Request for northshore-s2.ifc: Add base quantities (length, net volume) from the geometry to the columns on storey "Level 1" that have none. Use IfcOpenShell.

First a look at what the model holds.

```python
import ifcopenshell
import ifcopenshell.util.element
import ifcopenshell.util.unit

model = ifcopenshell.open("northshore-s2.ifc")
print(model.schema)
for unit_type in ("LENGTHUNIT", "AREAUNIT", "VOLUMEUNIT"):
    print(unit_type, ifcopenshell.util.unit.calculate_unit_scale(model, unit_type))
storey = next(s for s in model.by_type("IfcBuildingStorey") if s.Name == "Level 1")
columns = [e for e in ifcopenshell.util.element.get_decomposition(storey) if e.is_a("IfcColumn")]
for e in sorted(columns, key=lambda e: e.id()):
    print(e.id(), e.is_a(), e.Name, list(ifcopenshell.util.element.get_psets(e, qtos_only=True)), sep=" | ")
```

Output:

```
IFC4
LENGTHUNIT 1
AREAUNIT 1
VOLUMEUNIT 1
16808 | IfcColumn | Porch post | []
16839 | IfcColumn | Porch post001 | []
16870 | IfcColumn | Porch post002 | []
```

```python
import ifcopenshell
import ifcopenshell.api.pset
import ifcopenshell.geom
import ifcopenshell.util.element
import ifcopenshell.util.shape
import ifcopenshell.util.unit

model = ifcopenshell.open("northshore-s2.ifc")
unit_scale = ifcopenshell.util.unit.calculate_unit_scale(model)
volume_scale = ifcopenshell.util.unit.calculate_unit_scale(model, "VOLUMEUNIT")
settings = ifcopenshell.geom.settings()

storey = next(s for s in model.by_type("IfcBuildingStorey") if s.Name == "Level 1")
columns = [e for e in ifcopenshell.util.element.get_decomposition(storey) if e.is_a("IfcColumn")]

for e in sorted(columns, key=lambda e: e.id()):
    if ifcopenshell.util.element.get_psets(e, qtos_only=True, should_inherit=False):
        continue
    # Geometry comes back in metres, in the element's own axes.
    shape = ifcopenshell.geom.create_shape(settings, e)
    values = {
        "Length": ifcopenshell.util.shape.get_z(shape.geometry) / unit_scale,
        "NetVolume": ifcopenshell.util.shape.get_volume(shape.geometry) / volume_scale,
    }
    qto = ifcopenshell.api.pset.add_qto(model, product=e, name="Qto_ColumnBaseQuantities")
    ifcopenshell.api.pset.edit_qto(model, qto=qto, properties=values)
    print(e.id(), {k: round(v, 3) for k, v in values.items()})

model.write("northshore-s2_rev.ifc")
```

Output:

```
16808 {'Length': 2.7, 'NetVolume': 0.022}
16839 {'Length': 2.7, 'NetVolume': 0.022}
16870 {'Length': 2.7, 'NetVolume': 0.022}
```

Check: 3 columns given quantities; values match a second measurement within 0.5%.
